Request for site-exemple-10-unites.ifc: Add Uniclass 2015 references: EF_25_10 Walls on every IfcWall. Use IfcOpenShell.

First a look at what the model holds.

```python
import ifcopenshell

model = ifcopenshell.open("site-exemple-10-unites.ifc")
print(model.schema)
print("classifications:", [c.Name for c in model.by_type("IfcClassification")])
for ifc_class in ("IfcDoor", "IfcRoof", "IfcStair", "IfcWall", "IfcWindow"):
    print(ifc_class, len(model.by_type(ifc_class)))
```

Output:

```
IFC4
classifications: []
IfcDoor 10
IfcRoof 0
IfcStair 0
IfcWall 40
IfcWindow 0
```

```python
import ifcopenshell
import ifcopenshell.api.classification

model = ifcopenshell.open("site-exemple-10-unites.ifc")

system = ifcopenshell.api.classification.add_classification(model, classification="Uniclass 2015")

codes = {
    "IfcWall": ("EF_25_10", "Walls"),
}
for ifc_class, (code, name) in codes.items():
    products = model.by_type(ifc_class)
    ifcopenshell.api.classification.add_reference(
        model, products=products, classification=system, identification=code, name=name
    )
    print(code, len(products))

model.write("site-exemple-10-unites-out.ifc")
```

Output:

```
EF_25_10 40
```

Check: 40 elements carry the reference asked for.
